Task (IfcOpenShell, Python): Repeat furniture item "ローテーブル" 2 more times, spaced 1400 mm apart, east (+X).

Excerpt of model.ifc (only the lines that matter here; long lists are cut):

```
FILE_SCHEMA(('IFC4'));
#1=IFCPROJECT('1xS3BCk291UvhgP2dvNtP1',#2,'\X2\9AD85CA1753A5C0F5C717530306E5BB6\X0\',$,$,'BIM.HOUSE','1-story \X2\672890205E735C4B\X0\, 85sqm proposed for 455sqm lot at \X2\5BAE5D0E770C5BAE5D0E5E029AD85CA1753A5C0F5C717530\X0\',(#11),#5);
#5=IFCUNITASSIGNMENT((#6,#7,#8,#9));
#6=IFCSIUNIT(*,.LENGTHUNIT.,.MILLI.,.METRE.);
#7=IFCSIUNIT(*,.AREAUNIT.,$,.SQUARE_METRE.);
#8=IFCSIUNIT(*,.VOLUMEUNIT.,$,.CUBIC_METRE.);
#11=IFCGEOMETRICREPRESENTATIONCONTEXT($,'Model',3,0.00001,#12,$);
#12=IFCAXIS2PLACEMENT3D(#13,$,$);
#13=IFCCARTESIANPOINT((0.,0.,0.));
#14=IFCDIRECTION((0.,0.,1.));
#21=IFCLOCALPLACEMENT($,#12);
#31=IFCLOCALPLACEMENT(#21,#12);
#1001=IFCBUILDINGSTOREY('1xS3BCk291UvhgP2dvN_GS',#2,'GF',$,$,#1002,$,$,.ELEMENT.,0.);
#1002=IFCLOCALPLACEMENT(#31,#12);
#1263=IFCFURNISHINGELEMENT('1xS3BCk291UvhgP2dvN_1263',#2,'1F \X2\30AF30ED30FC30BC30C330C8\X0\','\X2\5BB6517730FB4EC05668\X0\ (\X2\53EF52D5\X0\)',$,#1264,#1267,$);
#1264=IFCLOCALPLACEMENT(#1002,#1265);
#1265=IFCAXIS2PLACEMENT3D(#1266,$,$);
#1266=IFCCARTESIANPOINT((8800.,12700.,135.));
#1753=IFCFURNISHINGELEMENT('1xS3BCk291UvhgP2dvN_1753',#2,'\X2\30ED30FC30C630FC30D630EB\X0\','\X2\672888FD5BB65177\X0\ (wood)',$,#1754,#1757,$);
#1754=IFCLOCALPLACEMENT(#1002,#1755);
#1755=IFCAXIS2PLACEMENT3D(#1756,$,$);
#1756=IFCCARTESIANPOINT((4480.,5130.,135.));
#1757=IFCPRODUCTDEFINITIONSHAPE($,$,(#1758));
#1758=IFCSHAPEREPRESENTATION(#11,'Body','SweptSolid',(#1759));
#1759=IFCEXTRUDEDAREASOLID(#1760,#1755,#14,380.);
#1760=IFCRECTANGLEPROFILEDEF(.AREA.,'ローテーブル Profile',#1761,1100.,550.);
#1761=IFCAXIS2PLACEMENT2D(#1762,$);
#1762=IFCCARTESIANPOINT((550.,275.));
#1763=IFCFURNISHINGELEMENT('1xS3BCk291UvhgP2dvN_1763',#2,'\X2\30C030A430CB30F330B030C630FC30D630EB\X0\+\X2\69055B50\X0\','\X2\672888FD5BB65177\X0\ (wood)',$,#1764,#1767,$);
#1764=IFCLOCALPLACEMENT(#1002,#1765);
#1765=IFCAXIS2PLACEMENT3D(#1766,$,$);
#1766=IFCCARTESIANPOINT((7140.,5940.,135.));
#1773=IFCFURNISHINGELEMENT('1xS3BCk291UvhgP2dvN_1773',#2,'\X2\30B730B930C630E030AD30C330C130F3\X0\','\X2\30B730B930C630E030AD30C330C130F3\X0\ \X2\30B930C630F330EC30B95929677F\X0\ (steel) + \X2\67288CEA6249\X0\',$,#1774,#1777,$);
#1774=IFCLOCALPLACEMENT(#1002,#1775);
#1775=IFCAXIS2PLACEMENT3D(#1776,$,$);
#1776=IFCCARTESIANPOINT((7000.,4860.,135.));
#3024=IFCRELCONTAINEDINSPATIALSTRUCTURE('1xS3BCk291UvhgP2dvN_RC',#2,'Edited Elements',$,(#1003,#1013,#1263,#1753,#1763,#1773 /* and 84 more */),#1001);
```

```python
import numpy as np
import ifcopenshell
import ifcopenshell.api.geometry
import ifcopenshell.api.root
import ifcopenshell.util.element
import ifcopenshell.util.placement

model = ifcopenshell.open("model.ifc")


def reuse_history(source, copy):
    """copy_class also copies each property set's owner history, people and application; keep the originals."""
    for rel in copy.IsDefinedBy:
        if rel.is_a("IfcRelDefinesByProperties") and (history := rel.RelatingPropertyDefinition.OwnerHistory):
            rel.RelatingPropertyDefinition.OwnerHistory = source.OwnerHistory
            ifcopenshell.util.element.remove_deep2(model, history)


source = model.by_guid("1xS3BCk291UvhgP2dvN_1753")
base = ifcopenshell.util.placement.get_local_placement(source.ObjectPlacement)
step = np.array([1.0, 0.0, 0.0]) * 1400.0

for i in range(1, 3):
    copy = ifcopenshell.api.root.copy_class(model, product=source)
    copy.Representation = ifcopenshell.util.element.copy_deep(
        model, source.Representation, exclude=["IfcGeometricRepresentationContext", "IfcRepresentationMap"]
    )
    reuse_history(source, copy)
    matrix = base.copy()
    matrix[:3, 3] += i * step
    print("added at", matrix[:3, 3].round(3) + 0.0)
    ifcopenshell.api.geometry.edit_object_placement(model, product=copy, matrix=matrix, is_si=False)

model.write("model_rev.ifc")
```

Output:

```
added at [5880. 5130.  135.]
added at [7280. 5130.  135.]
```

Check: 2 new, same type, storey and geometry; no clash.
